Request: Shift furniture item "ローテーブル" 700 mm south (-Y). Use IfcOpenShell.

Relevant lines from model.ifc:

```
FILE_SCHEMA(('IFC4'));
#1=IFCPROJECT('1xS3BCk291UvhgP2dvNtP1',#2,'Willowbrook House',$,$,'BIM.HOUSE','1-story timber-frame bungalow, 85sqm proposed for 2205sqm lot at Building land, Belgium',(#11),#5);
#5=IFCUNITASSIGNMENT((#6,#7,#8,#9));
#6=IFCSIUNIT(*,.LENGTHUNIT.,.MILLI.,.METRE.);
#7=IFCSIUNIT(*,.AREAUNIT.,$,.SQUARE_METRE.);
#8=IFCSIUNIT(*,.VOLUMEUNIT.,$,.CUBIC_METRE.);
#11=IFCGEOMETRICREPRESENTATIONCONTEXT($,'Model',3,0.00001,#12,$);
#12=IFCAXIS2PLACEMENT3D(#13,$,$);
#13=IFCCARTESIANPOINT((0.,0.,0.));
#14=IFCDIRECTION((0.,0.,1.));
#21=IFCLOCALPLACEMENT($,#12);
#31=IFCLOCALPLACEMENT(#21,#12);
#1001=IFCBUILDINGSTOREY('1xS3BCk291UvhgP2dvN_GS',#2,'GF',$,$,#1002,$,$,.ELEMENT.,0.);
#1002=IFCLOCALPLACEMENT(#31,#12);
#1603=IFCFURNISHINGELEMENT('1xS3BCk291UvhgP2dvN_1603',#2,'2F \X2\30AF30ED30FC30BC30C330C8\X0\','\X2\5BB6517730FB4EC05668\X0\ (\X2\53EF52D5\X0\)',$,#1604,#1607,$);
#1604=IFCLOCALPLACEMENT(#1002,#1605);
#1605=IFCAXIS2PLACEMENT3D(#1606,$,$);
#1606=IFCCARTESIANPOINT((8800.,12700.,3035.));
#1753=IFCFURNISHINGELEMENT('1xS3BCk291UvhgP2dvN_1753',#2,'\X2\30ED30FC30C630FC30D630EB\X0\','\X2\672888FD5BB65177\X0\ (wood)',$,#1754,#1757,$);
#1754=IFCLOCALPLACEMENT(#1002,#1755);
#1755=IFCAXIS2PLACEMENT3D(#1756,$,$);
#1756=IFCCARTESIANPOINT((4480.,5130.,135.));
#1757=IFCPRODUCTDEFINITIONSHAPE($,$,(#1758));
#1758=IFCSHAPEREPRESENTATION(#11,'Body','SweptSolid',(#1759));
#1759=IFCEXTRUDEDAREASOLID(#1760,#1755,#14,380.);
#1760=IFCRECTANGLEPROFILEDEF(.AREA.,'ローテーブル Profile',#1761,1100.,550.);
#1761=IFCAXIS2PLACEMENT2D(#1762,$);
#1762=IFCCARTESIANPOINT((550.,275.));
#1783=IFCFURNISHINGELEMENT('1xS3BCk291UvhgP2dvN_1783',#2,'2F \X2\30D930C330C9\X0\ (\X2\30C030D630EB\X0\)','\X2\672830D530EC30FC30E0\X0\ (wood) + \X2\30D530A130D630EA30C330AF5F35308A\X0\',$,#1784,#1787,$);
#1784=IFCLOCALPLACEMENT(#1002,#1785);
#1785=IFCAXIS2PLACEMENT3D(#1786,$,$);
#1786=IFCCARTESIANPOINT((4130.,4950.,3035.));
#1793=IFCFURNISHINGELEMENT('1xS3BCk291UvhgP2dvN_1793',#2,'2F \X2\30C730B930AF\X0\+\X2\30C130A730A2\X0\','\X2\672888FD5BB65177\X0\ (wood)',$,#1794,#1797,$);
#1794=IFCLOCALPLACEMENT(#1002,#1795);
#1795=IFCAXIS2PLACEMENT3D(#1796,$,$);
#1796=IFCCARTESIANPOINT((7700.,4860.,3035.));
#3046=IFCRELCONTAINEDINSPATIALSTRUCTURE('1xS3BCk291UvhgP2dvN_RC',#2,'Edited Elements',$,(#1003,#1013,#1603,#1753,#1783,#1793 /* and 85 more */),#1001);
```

```python
import ifcopenshell
import ifcopenshell.api.geometry
import ifcopenshell.util.placement
import ifcopenshell.util.unit

model = ifcopenshell.open("model.ifc")
unit_scale = ifcopenshell.util.unit.calculate_unit_scale(model)

item = model.by_guid("1xS3BCk291UvhgP2dvN_1753")
matrix = ifcopenshell.util.placement.get_local_placement(item.ObjectPlacement)
matrix[1, 3] -= 0.7 / unit_scale
ifcopenshell.api.geometry.edit_object_placement(model, product=item, matrix=matrix, is_si=False)

print(ifcopenshell.util.placement.get_local_placement(item.ObjectPlacement).round(3) + 0.0)

model.write("model-out.ifc")
```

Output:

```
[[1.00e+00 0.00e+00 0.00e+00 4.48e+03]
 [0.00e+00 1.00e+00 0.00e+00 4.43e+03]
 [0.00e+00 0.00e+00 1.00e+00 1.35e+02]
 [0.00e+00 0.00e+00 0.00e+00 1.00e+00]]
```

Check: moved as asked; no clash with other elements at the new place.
